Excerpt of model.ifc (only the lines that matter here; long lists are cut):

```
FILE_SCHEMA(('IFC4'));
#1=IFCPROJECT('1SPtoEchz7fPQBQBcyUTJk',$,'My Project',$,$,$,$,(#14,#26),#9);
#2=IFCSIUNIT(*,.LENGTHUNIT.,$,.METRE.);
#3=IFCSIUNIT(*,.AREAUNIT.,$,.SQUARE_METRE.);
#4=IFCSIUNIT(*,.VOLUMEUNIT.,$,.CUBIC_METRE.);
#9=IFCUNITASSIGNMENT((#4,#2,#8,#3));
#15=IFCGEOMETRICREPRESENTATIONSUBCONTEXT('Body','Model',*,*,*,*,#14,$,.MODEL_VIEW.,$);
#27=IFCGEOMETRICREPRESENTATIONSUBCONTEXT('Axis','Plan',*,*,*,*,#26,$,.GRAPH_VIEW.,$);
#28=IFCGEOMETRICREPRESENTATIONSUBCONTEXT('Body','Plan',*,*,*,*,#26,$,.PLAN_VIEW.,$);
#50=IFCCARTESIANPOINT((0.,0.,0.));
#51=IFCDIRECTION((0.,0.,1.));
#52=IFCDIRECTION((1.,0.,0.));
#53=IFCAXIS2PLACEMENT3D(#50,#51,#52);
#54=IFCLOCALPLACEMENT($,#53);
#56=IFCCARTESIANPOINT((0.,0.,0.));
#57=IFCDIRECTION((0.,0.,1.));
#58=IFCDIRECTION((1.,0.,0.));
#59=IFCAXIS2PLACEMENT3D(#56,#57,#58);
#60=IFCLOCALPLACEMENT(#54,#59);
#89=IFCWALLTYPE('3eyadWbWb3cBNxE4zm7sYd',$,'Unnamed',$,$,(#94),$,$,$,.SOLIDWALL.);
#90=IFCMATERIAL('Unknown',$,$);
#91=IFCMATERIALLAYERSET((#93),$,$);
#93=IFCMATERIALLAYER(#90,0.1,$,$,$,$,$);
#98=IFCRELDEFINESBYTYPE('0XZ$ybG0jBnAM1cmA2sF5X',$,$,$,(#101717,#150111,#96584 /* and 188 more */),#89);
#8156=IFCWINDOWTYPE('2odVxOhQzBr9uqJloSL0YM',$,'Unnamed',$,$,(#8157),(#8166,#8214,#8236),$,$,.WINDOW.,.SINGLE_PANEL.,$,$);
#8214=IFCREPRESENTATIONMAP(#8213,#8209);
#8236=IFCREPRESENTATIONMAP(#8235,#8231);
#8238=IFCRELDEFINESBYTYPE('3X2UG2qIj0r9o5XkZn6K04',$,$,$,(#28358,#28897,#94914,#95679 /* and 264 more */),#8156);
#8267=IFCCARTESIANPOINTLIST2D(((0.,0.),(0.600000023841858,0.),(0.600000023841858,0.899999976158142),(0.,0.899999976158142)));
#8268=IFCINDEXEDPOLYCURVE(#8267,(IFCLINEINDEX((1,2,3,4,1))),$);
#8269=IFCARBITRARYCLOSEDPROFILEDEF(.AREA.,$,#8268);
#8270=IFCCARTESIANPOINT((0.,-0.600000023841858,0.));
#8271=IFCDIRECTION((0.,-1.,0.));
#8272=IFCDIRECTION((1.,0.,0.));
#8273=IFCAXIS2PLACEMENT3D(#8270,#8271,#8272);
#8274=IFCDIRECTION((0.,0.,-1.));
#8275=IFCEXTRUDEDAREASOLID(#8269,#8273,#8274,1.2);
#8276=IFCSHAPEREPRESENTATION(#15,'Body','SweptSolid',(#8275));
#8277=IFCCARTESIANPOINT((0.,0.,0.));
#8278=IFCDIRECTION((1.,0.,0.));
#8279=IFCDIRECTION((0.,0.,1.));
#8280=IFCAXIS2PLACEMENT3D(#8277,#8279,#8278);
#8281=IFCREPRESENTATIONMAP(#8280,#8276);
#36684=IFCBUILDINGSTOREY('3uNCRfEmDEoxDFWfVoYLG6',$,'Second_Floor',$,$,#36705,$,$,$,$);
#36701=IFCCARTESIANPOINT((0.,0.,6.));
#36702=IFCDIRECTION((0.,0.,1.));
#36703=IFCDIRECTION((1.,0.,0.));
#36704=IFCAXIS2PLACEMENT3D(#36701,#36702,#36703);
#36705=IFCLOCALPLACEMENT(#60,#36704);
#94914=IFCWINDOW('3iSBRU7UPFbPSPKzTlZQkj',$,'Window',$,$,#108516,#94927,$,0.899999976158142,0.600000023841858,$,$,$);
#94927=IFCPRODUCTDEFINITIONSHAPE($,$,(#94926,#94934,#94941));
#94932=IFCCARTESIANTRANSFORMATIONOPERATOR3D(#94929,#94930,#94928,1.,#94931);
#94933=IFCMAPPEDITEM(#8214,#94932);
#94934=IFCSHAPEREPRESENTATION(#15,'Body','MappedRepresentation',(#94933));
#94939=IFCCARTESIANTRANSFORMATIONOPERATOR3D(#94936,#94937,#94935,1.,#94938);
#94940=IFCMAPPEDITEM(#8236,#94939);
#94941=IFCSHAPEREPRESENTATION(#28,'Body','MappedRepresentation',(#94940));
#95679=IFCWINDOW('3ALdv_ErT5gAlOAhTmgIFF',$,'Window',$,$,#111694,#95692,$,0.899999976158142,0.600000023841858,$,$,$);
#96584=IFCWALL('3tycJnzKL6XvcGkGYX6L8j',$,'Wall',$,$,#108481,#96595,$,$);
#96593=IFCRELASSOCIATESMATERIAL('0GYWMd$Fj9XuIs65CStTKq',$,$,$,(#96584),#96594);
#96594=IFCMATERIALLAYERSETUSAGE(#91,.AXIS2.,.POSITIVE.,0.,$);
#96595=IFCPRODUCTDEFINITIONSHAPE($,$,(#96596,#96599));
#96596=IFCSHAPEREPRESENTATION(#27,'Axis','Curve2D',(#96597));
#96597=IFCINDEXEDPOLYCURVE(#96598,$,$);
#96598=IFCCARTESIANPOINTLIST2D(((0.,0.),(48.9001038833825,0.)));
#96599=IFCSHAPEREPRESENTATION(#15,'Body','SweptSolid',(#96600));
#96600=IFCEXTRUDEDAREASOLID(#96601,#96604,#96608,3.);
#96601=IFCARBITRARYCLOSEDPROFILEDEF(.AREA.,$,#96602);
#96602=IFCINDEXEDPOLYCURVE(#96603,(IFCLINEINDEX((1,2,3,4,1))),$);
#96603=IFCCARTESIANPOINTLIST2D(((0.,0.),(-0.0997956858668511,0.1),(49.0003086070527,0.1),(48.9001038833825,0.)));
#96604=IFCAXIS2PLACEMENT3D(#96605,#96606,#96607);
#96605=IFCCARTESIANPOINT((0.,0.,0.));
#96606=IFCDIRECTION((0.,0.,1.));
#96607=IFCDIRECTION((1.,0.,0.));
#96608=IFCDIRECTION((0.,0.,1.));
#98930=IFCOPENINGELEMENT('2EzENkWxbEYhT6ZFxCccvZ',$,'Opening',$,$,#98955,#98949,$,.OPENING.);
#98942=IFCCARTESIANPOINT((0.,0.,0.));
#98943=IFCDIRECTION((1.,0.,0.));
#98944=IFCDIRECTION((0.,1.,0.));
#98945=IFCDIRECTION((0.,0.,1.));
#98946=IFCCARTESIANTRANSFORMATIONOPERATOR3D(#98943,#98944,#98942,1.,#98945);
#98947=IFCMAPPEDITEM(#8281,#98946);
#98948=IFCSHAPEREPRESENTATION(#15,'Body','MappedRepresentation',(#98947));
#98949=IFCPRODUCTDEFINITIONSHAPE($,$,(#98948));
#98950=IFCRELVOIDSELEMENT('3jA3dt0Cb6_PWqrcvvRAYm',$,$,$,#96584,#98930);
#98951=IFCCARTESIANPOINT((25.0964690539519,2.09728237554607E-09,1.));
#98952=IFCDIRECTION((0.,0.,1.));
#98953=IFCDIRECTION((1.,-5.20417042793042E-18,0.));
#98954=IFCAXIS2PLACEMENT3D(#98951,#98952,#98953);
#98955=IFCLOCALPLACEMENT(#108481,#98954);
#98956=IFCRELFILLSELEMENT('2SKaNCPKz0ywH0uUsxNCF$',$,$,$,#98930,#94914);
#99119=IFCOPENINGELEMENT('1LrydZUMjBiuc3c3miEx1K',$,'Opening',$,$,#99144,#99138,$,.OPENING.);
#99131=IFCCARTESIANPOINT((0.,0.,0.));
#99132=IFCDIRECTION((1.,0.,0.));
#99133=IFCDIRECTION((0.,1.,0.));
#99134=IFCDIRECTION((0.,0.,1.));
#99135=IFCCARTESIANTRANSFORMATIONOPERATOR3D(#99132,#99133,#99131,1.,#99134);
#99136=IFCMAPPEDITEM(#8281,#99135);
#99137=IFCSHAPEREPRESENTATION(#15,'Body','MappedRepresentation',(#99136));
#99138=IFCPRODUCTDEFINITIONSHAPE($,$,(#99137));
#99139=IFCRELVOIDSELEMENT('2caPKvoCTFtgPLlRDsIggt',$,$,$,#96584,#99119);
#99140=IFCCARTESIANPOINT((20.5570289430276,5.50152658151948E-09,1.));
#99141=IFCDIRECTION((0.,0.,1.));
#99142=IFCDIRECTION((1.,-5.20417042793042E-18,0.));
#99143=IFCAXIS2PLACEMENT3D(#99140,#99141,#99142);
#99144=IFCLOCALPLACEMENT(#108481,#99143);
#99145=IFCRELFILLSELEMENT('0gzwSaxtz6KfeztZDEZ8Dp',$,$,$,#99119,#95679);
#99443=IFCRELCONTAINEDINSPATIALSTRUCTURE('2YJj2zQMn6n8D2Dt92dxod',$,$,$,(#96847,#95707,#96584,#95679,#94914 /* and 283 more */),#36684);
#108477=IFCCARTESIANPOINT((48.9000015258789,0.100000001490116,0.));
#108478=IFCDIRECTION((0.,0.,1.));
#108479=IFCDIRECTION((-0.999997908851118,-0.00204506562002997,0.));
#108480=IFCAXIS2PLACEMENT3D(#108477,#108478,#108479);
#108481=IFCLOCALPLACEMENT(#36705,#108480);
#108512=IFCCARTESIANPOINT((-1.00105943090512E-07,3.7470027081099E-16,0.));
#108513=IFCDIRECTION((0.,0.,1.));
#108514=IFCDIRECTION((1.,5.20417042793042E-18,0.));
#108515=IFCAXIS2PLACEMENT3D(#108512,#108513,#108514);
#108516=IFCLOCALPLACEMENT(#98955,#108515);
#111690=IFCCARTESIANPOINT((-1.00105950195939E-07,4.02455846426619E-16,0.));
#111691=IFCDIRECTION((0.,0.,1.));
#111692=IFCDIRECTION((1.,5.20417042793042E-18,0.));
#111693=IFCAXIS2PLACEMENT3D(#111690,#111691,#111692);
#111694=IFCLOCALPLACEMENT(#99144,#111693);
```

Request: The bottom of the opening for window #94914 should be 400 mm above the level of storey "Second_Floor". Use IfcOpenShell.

```python
import numpy as np
import ifcopenshell
import ifcopenshell.api.geometry
import ifcopenshell.geom
import ifcopenshell.util.element
import ifcopenshell.util.placement
import ifcopenshell.util.shape
import ifcopenshell.util.unit

model = ifcopenshell.open("model.ifc")
unit_scale = ifcopenshell.util.unit.calculate_unit_scale(model)

window = model.by_guid("3iSBRU7UPFbPSPKzTlZQkj")
opening = window.FillsVoids[0].RelatingOpeningElement
storey = ifcopenshell.util.element.get_container(window, ifc_class="IfcBuildingStorey")
level = ifcopenshell.util.placement.get_local_placement(storey.ObjectPlacement)[2, 3]

# The opening's origin need not be at the sill, so measure its lowest point.
shape = ifcopenshell.geom.create_shape(ifcopenshell.geom.settings(), opening)
bottom = ifcopenshell.util.shape.get_shape_bottom_elevation(shape, shape.geometry) / unit_scale
dz = level + 0.4 - bottom

shift = np.array([0.0, 0.0, dz])
# The window is placed relative to its opening, so it follows when the opening moves.
matrix = ifcopenshell.util.placement.get_local_placement(opening.ObjectPlacement)
matrix[:3, 3] += shift
ifcopenshell.api.geometry.edit_object_placement(
    model, product=opening, matrix=matrix, is_si=False, should_transform_children=True
)

print(f"moved by {dz * unit_scale:+.3f} m")

model.write("model_updated.ifc")
```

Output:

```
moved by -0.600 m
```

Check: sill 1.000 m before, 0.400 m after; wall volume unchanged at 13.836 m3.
